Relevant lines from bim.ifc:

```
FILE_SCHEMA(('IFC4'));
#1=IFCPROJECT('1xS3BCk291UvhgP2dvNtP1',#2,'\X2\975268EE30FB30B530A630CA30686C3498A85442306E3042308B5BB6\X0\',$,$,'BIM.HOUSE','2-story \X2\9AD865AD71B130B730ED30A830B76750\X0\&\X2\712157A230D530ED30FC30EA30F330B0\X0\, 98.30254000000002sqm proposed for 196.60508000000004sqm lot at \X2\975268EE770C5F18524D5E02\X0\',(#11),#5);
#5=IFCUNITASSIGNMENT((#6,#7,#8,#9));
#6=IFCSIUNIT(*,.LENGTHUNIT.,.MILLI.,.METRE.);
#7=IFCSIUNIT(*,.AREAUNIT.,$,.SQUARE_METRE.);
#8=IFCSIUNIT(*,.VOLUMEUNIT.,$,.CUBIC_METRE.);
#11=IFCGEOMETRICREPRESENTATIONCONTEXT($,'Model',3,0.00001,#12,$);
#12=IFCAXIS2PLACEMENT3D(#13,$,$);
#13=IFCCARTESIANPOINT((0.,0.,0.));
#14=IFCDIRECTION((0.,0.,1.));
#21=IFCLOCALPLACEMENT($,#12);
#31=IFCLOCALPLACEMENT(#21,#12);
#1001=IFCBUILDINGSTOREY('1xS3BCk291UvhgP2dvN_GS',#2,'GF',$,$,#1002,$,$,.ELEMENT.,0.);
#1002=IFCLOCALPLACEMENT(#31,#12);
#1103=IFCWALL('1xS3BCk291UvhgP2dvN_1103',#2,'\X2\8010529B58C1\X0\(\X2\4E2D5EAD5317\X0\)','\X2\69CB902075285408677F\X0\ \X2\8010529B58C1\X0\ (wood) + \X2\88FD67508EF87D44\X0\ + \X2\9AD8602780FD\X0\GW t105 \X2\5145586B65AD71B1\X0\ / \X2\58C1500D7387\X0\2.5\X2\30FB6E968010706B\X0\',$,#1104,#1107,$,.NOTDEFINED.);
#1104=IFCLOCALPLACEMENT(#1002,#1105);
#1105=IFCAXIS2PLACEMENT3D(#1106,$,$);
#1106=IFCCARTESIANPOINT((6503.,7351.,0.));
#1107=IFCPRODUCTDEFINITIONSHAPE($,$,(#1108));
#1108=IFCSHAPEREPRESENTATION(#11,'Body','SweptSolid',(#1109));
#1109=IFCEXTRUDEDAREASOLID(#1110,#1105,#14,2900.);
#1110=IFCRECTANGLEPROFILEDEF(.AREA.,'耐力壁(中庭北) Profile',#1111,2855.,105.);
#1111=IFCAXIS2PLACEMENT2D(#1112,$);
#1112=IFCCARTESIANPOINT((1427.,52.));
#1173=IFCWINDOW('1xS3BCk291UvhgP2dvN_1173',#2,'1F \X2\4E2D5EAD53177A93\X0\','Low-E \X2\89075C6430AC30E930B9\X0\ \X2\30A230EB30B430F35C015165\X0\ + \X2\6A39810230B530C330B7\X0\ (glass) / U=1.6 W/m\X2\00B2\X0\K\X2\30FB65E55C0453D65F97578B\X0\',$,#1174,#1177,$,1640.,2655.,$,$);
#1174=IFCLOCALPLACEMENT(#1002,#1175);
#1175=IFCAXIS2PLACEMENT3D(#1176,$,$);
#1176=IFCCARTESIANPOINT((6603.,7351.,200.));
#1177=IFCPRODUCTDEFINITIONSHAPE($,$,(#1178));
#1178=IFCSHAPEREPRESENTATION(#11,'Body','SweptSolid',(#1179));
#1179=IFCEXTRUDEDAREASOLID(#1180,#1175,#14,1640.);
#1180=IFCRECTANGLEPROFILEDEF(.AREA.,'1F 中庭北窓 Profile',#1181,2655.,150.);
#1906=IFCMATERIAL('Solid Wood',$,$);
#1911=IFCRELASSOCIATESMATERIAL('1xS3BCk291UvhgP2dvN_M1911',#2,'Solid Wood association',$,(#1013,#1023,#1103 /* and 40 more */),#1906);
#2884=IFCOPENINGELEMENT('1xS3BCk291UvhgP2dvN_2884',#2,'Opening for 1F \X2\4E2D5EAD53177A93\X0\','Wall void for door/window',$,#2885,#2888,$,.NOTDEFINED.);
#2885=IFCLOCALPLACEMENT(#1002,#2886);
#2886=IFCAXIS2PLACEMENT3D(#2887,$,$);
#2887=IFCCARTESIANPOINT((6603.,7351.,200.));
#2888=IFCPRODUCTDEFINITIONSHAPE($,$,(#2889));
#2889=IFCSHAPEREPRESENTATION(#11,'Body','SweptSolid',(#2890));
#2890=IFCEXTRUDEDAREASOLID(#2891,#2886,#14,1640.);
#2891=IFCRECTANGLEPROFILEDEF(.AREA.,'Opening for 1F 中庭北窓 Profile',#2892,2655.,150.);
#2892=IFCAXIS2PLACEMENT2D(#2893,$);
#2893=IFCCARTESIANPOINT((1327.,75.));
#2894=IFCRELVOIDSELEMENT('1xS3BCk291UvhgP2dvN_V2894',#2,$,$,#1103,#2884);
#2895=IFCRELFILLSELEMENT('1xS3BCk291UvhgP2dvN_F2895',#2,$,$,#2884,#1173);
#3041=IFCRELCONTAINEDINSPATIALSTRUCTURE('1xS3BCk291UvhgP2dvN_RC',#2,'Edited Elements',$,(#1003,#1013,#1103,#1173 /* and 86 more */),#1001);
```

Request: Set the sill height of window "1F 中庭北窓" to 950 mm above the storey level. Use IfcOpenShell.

```python
import numpy as np
import ifcopenshell
import ifcopenshell.api.geometry
import ifcopenshell.geom
import ifcopenshell.util.element
import ifcopenshell.util.placement
import ifcopenshell.util.shape
import ifcopenshell.util.unit

model = ifcopenshell.open("bim.ifc")
unit_scale = ifcopenshell.util.unit.calculate_unit_scale(model)

window = model.by_guid("1xS3BCk291UvhgP2dvN_1173")
opening = window.FillsVoids[0].RelatingOpeningElement
storey = ifcopenshell.util.element.get_container(window, ifc_class="IfcBuildingStorey")
level = ifcopenshell.util.placement.get_local_placement(storey.ObjectPlacement)[2, 3]

# The opening's origin need not be at the sill, so measure its lowest point.
shape = ifcopenshell.geom.create_shape(ifcopenshell.geom.settings(), opening)
bottom = ifcopenshell.util.shape.get_shape_bottom_elevation(shape, shape.geometry) / unit_scale
dz = level + 950.0 - bottom

shift = np.array([0.0, 0.0, dz])
# The window is not placed relative to its opening, so move both.
for product in (opening, window):
    matrix = ifcopenshell.util.placement.get_local_placement(product.ObjectPlacement)
    matrix[:3, 3] += shift
    ifcopenshell.api.geometry.edit_object_placement(model, product=product, matrix=matrix, is_si=False)

print(f"moved by {dz * unit_scale:+.3f} m")

model.write("bim_edited.ifc")
```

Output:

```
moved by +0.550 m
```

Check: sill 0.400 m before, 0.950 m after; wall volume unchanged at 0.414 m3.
